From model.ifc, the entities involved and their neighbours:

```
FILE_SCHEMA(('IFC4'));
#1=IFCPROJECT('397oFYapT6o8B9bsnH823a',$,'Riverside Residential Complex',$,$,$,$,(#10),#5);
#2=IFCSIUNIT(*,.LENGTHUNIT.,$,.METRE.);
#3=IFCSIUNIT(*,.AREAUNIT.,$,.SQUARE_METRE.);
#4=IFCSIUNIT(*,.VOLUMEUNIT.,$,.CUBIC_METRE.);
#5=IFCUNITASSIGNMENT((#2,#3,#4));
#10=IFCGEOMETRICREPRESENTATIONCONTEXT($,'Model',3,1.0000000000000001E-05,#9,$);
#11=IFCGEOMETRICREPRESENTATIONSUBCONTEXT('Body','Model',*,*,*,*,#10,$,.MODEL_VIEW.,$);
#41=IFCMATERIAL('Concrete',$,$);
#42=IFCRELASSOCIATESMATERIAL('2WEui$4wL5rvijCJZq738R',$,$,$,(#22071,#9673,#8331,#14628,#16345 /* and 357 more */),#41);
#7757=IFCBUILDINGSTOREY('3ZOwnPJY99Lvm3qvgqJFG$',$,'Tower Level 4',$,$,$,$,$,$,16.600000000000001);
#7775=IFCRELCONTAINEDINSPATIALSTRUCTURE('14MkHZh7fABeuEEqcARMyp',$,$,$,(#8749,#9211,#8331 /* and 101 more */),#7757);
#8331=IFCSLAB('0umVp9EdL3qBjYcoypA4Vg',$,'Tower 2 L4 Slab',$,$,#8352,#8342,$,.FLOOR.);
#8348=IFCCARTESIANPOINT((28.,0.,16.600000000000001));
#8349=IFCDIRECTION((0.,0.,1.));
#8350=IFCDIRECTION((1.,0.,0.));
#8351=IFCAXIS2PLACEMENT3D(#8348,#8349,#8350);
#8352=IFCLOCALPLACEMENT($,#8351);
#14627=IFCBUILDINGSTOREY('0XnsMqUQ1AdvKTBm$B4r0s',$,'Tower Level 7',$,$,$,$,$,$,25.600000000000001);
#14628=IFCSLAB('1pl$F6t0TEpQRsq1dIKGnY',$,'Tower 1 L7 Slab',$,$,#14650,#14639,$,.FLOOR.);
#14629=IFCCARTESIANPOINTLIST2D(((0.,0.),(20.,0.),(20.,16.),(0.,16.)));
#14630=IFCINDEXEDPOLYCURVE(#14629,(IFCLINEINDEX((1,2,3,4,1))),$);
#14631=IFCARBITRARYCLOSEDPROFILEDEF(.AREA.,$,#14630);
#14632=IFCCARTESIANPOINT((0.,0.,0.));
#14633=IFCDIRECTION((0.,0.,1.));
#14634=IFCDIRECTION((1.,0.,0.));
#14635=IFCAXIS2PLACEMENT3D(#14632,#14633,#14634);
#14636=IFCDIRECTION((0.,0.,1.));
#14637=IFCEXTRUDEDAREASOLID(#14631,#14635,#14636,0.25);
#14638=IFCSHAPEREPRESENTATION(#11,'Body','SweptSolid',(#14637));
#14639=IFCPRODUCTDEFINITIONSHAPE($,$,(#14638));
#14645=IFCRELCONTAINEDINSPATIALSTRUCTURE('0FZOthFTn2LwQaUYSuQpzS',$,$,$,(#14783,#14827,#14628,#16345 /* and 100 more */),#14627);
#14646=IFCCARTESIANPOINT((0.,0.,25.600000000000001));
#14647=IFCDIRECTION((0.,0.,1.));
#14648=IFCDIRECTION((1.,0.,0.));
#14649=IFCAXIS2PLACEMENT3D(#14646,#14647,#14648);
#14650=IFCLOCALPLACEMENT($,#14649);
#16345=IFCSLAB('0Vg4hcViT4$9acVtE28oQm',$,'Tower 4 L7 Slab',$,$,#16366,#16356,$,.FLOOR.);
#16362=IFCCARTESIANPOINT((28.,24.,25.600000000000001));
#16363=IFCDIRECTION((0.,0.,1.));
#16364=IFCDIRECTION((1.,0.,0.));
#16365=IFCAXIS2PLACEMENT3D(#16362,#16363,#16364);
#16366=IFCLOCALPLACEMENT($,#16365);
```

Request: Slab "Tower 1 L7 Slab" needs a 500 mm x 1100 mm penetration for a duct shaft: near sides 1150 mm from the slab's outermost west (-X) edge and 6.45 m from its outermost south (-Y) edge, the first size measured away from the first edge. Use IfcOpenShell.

```python
import numpy as np
import ifcopenshell
import ifcopenshell.api.feature
import ifcopenshell.api.geometry
import ifcopenshell.api.root
import ifcopenshell.geom
import ifcopenshell.util.placement
import ifcopenshell.util.representation
import ifcopenshell.util.shape
import ifcopenshell.util.unit

model = ifcopenshell.open("model.ifc")
unit_scale = ifcopenshell.util.unit.calculate_unit_scale(model)
settings = ifcopenshell.geom.settings()


def volume(element):
    """Net volume in cubic metres, openings subtracted."""
    shape = ifcopenshell.geom.create_shape(settings, element)
    return ifcopenshell.util.shape.get_volume(shape.geometry)


slab = model.by_guid("1pl$F6t0TEpQRsq1dIKGnY")
before = volume(slab)

# Extent in the slab's own axes, in metres. The edges named are its -X and -Y sides.
slab_shape = ifcopenshell.geom.create_shape(settings, slab)
vertices = ifcopenshell.util.shape.get_vertices(slab_shape.geometry)
x_min, y_min, bottom = vertices.min(axis=0)
top = vertices[:, 2].max()

opening = ifcopenshell.api.root.create_entity(model, ifc_class="IfcOpeningElement", name="Duct shaft opening", predefined_type="OPENING")
context = ifcopenshell.util.representation.get_context(model, "Model", "Body", "MODEL_VIEW")
width, depth = 0.5, 1.1
outline = [(0.0, 0.0), (width, 0.0), (width, depth), (0.0, depth), (0.0, 0.0)]
# Overshoot both faces by 50 mm so the cut is clean.
shape = ifcopenshell.api.geometry.add_slab_representation(
    model, context=context, depth=top - bottom + 0.1, polyline=outline
)
ifcopenshell.api.geometry.assign_representation(model, product=opening, representation=shape)

matrix = ifcopenshell.util.placement.get_local_placement(slab.ObjectPlacement)
matrix[:, 3] = matrix @ np.append(np.array([x_min + 1.15, y_min + 6.45, bottom - 0.05]) / unit_scale, 1.0)
ifcopenshell.api.geometry.edit_object_placement(model, product=opening, matrix=matrix, is_si=False)
ifcopenshell.api.feature.add_feature(model, feature=opening, element=slab)

after = volume(slab)

print(f"slab volume {before:.3f} -> {after:.3f} m3")

model.write("model_edited.ifc")
```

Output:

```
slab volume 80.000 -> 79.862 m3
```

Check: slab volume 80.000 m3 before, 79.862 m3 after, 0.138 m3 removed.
